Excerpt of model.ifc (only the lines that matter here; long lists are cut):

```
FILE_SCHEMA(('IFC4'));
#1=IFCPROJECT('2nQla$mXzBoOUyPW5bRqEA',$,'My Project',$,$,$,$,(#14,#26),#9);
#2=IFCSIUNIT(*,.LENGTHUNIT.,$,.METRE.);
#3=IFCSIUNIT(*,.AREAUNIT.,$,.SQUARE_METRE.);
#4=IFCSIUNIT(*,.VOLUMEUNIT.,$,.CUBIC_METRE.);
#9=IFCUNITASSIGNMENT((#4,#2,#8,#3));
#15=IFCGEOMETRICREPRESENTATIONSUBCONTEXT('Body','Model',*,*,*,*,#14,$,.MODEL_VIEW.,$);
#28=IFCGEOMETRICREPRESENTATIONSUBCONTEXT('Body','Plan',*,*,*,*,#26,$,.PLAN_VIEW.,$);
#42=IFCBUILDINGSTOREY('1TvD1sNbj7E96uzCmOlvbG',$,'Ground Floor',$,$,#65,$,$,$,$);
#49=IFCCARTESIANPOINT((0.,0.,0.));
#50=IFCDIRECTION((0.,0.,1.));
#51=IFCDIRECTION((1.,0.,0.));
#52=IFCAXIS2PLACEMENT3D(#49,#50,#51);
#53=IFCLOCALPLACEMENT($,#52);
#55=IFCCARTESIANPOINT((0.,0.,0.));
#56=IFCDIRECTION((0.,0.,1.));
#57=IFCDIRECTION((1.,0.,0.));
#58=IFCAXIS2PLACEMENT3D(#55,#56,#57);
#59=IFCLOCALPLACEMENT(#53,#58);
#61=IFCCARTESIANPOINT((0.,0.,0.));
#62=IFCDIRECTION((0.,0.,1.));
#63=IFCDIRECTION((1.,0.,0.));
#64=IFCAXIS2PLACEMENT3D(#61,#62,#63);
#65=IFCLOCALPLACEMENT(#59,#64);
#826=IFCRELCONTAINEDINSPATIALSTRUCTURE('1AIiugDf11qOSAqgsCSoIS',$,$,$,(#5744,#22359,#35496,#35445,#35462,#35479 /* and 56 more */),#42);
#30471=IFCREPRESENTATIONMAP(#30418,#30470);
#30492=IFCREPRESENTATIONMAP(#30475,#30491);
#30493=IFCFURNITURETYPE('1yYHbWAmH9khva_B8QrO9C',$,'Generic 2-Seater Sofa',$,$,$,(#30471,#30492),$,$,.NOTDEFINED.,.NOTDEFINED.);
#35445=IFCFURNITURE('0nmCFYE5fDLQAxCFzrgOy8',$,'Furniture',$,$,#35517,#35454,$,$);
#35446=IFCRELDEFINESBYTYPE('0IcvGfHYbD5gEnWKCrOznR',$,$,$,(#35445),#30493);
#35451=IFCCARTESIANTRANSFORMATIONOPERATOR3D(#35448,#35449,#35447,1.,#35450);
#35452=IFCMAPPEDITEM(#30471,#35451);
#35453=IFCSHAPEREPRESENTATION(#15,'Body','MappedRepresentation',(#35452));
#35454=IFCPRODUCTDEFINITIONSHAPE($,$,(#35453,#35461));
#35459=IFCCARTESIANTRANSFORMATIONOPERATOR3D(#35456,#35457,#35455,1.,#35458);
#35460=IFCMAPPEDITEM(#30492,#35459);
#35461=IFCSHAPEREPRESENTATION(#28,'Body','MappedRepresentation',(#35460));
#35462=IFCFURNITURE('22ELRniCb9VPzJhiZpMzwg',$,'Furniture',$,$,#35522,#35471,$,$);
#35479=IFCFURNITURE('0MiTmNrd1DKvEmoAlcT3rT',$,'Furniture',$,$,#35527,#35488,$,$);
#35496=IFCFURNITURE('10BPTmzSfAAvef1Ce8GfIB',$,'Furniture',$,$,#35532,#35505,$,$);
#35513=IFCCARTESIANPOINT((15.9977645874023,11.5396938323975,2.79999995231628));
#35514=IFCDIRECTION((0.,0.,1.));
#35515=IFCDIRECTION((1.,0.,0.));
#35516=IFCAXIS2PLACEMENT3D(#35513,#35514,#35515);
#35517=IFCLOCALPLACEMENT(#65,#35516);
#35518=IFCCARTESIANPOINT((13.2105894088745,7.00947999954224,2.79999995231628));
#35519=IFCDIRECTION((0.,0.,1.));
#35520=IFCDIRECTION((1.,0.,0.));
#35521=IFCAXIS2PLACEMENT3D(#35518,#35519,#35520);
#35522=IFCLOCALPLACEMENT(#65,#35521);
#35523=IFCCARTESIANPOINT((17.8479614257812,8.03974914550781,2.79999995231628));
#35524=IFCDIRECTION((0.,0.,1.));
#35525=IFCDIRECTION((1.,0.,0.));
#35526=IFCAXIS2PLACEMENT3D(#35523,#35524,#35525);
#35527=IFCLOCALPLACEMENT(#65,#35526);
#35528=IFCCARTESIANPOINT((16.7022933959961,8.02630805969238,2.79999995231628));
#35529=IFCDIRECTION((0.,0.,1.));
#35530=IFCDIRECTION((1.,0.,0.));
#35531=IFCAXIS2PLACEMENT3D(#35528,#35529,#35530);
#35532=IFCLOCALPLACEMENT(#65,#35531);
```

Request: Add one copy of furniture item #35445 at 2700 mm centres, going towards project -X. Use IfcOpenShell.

```python
import numpy as np
import ifcopenshell
import ifcopenshell.api.geometry
import ifcopenshell.api.root
import ifcopenshell.util.element
import ifcopenshell.util.placement

model = ifcopenshell.open("model.ifc")

source = model.by_guid("0nmCFYE5fDLQAxCFzrgOy8")
base = ifcopenshell.util.placement.get_local_placement(source.ObjectPlacement)
step = np.array([-1.0, 0.0, 0.0]) * 2.7

for i in range(1, 2):
    copy = ifcopenshell.api.root.copy_class(model, product=source)
    copy.Representation = ifcopenshell.util.element.copy_deep(
        model, source.Representation, exclude=["IfcGeometricRepresentationContext", "IfcRepresentationMap"]
    )
    matrix = base.copy()
    matrix[:3, 3] += i * step
    print("added at", matrix[:3, 3].round(3) + 0.0)
    ifcopenshell.api.geometry.edit_object_placement(model, product=copy, matrix=matrix, is_si=False)

model.write("model_edited.ifc")
```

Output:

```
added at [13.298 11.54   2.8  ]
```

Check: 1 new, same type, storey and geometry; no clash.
